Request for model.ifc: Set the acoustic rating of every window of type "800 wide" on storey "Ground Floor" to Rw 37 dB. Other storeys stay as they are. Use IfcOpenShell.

First a look at what the model holds.

```python
import ifcopenshell
import ifcopenshell.util.element

model = ifcopenshell.open("model.ifc")
print(model.schema)
storey = next(s for s in model.by_type("IfcBuildingStorey") if s.Name == "Ground Floor")
windows = [e for e in ifcopenshell.util.element.get_decomposition(storey) if e.is_a("IfcWindow")]
seen = {}
for e in windows:
    element_type = ifcopenshell.util.element.get_type(e)
    key = (element_type.Name if element_type != e and element_type else None, ifcopenshell.util.element.get_pset(e, "Pset_WindowCommon", "AcousticRating"))
    seen[key] = seen.get(key, 0) + 1
for (name, value), count in sorted(seen.items(), key=str):
    print(count, "x", name, "|", value)
```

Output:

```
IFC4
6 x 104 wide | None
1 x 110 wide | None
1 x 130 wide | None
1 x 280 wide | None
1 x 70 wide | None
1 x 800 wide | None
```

```python
import ifcopenshell
import ifcopenshell.api.pset
import ifcopenshell.util.element

model = ifcopenshell.open("model.ifc")

storey = next(s for s in model.by_type("IfcBuildingStorey") if s.Name == "Ground Floor")
windows = [e for e in ifcopenshell.util.element.get_decomposition(storey) if e.is_a("IfcWindow")]

count = 0
for e in windows:
    element_type = ifcopenshell.util.element.get_type(e)
    if element_type in (None, e) or element_type.Name != "800 wide":
        continue
    # add_pset returns the element's existing set when there is one.
    pset = ifcopenshell.api.pset.add_pset(model, product=e, name="Pset_WindowCommon")
    ifcopenshell.api.pset.edit_pset(model, pset=pset, properties={"AcousticRating": "Rw 37 dB"})
    count += 1

print(count, "windows updated")

model.write("model_v2.ifc")
```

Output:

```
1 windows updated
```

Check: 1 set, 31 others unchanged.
